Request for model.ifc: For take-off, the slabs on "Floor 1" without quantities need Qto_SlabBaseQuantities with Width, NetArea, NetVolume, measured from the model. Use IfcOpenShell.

First a look at what the model holds.

```python
import ifcopenshell
import ifcopenshell.util.element
import ifcopenshell.util.unit

model = ifcopenshell.open("model.ifc")
print(model.schema)
for unit_type in ("LENGTHUNIT", "AREAUNIT", "VOLUMEUNIT"):
    print(unit_type, ifcopenshell.util.unit.calculate_unit_scale(model, unit_type))
storey = next(s for s in model.by_type("IfcBuildingStorey") if s.Name == "Floor 1")
slabs = [e for e in ifcopenshell.util.element.get_decomposition(storey) if e.is_a("IfcSlab")]
for e in sorted(slabs, key=lambda e: e.id()):
    print(e.id(), e.is_a(), e.Name, list(ifcopenshell.util.element.get_psets(e, qtos_only=True)), sep=" | ")
```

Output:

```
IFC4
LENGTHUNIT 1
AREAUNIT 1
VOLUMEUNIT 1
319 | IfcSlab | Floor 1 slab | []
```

```python
import ifcopenshell
import ifcopenshell.api.pset
import ifcopenshell.geom
import ifcopenshell.util.element
import ifcopenshell.util.shape
import ifcopenshell.util.unit

model = ifcopenshell.open("model.ifc")
unit_scale = ifcopenshell.util.unit.calculate_unit_scale(model)
area_scale = ifcopenshell.util.unit.calculate_unit_scale(model, "AREAUNIT")
volume_scale = ifcopenshell.util.unit.calculate_unit_scale(model, "VOLUMEUNIT")
settings = ifcopenshell.geom.settings()

storey = next(s for s in model.by_type("IfcBuildingStorey") if s.Name == "Floor 1")
slabs = [e for e in ifcopenshell.util.element.get_decomposition(storey) if e.is_a("IfcSlab")]

for e in sorted(slabs, key=lambda e: e.id()):
    if ifcopenshell.util.element.get_psets(e, qtos_only=True, should_inherit=False):
        continue
    # Geometry comes back in metres, in the element's own axes.
    shape = ifcopenshell.geom.create_shape(settings, e)
    values = {
        "Width": ifcopenshell.util.shape.get_z(shape.geometry) / unit_scale,
        "NetArea": ifcopenshell.util.shape.get_footprint_area(shape.geometry) / area_scale,
        "NetVolume": ifcopenshell.util.shape.get_volume(shape.geometry) / volume_scale,
    }
    qto = ifcopenshell.api.pset.add_qto(model, product=e, name="Qto_SlabBaseQuantities")
    ifcopenshell.api.pset.edit_qto(model, qto=qto, properties=values)
    print(e.id(), {k: round(v, 3) for k, v in values.items()})

model.write("model_rev.ifc")
```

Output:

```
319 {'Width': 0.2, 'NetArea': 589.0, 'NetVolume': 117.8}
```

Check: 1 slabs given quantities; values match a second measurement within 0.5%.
